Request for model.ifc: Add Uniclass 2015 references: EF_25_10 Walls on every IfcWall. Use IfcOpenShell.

First a look at what the model holds.

```python
import ifcopenshell

model = ifcopenshell.open("model.ifc")
print(model.schema)
print("classifications:", [c.Name for c in model.by_type("IfcClassification")])
for ifc_class in ("IfcDoor", "IfcRoof", "IfcStair", "IfcWall", "IfcWindow"):
    print(ifc_class, len(model.by_type(ifc_class)))
```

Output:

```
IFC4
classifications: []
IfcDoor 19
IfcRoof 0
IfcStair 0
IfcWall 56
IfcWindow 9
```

```python
import ifcopenshell
import ifcopenshell.api.classification

model = ifcopenshell.open("model.ifc")

system = ifcopenshell.api.classification.add_classification(model, classification="Uniclass 2015")

codes = {
    "IfcWall": ("EF_25_10", "Walls"),
}
for ifc_class, (code, name) in codes.items():
    products = model.by_type(ifc_class)
    ifcopenshell.api.classification.add_reference(
        model, products=products, classification=system, identification=code, name=name
    )
    print(code, len(products))

model.write("model_v2.ifc")
```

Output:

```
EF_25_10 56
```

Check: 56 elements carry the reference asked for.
